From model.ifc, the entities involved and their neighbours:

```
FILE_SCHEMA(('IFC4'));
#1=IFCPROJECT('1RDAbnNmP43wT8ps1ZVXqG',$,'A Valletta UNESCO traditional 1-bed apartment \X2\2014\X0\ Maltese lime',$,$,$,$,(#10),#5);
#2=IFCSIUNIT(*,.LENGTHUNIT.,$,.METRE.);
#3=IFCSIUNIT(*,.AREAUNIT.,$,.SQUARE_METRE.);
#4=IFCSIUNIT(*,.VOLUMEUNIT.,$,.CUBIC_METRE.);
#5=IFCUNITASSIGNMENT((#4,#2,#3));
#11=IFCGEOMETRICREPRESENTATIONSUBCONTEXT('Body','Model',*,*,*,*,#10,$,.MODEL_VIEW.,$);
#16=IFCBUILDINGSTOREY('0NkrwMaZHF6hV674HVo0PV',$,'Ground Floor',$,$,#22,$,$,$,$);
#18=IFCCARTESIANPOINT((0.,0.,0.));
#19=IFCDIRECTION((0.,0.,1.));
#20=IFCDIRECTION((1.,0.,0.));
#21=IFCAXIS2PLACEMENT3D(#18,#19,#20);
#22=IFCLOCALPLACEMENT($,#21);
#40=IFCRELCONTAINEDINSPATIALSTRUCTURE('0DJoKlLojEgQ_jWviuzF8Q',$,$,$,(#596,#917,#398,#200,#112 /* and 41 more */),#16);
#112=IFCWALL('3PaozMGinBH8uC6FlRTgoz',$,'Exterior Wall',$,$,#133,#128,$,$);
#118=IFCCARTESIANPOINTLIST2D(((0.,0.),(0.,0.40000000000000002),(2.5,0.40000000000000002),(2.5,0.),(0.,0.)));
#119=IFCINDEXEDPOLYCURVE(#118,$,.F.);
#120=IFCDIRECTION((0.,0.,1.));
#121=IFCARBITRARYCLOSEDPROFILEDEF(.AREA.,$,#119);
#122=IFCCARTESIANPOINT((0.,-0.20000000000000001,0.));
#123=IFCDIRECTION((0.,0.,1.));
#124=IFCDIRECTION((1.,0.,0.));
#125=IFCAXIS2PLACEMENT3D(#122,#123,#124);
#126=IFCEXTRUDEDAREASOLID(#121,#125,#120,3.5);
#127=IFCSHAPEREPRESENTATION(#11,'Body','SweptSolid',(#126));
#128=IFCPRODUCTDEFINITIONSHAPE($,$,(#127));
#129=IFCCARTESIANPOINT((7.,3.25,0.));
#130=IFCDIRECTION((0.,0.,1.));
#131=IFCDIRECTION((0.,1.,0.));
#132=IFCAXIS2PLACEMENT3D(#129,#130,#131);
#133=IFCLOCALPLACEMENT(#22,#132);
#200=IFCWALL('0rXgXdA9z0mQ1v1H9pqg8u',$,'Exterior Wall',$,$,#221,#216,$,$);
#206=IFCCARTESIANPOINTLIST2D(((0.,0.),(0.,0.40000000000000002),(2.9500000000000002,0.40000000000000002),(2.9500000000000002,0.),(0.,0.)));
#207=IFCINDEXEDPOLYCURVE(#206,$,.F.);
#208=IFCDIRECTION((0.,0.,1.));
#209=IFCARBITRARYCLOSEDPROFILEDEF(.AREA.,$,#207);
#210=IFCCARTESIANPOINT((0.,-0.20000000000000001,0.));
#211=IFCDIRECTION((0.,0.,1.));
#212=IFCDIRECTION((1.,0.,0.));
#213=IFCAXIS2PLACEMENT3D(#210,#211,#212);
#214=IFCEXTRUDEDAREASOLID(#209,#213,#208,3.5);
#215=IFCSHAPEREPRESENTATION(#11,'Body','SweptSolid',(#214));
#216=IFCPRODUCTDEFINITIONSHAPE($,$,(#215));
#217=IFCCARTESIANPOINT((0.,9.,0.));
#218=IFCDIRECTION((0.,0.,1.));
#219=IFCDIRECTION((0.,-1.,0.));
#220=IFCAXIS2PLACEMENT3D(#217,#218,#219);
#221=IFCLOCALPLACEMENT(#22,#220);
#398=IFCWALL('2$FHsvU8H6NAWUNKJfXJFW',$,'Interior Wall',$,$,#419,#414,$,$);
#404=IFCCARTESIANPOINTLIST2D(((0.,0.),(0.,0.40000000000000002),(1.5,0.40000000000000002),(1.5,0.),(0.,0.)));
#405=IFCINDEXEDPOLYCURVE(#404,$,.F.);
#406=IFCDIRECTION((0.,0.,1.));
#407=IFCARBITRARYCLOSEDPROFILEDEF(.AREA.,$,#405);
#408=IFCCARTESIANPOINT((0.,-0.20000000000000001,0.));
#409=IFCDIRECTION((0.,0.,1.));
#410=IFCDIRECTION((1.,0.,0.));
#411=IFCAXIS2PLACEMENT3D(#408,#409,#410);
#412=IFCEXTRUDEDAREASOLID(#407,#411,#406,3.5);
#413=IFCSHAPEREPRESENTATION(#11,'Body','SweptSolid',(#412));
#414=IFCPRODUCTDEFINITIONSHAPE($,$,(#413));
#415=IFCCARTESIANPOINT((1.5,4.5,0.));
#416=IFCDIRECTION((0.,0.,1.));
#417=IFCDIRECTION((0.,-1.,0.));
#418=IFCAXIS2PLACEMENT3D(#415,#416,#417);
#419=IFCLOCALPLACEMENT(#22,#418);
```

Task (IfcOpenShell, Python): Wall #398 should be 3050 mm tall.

```python
import ifcopenshell
import ifcopenshell.geom
import ifcopenshell.util.representation
import ifcopenshell.util.shape
import ifcopenshell.util.unit

model = ifcopenshell.open("model.ifc")
unit_scale = ifcopenshell.util.unit.calculate_unit_scale(model)
settings = ifcopenshell.geom.settings()


def volume(element):
    """Net volume in cubic metres, openings subtracted."""
    shape = ifcopenshell.geom.create_shape(settings, element)
    return ifcopenshell.util.shape.get_volume(shape.geometry)


wall = model.by_guid("2$FHsvU8H6NAWUNKJfXJFW")
before = volume(wall)

body = ifcopenshell.util.representation.get_representation(wall, "Model", "Body")
solid = body.Items[0]
old_height = solid.Depth
solid.Depth = 3.05 / unit_scale
after = volume(wall)

print(f"height {old_height:g} -> {solid.Depth:g}, volume {before:.3f} -> {after:.3f} m3")

model.write("model_edited.ifc")
```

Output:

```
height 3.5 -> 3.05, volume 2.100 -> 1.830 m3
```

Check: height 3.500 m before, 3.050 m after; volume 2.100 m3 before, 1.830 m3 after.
